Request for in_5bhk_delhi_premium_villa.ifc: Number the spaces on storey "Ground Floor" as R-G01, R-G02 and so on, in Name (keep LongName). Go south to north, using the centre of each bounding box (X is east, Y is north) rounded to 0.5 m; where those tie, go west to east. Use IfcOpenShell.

First a look at what the model holds.

```python
import ifcopenshell
import ifcopenshell.util.element
import ifcopenshell.util.placement

model = ifcopenshell.open("in_5bhk_delhi_premium_villa.ifc")
print(model.schema)
storey = next(s for s in model.by_type("IfcBuildingStorey") if s.Name == "Ground Floor")
spaces = [e for e in ifcopenshell.util.element.get_decomposition(storey) if e.is_a("IfcSpace")]
for e in sorted(spaces, key=lambda e: e.id()):
    origin = ifcopenshell.util.placement.get_local_placement(e.ObjectPlacement)[:3, 3]
    print(e.id(), e.Name, e.LongName, origin.round(2) + 0.0, sep=" | ")
```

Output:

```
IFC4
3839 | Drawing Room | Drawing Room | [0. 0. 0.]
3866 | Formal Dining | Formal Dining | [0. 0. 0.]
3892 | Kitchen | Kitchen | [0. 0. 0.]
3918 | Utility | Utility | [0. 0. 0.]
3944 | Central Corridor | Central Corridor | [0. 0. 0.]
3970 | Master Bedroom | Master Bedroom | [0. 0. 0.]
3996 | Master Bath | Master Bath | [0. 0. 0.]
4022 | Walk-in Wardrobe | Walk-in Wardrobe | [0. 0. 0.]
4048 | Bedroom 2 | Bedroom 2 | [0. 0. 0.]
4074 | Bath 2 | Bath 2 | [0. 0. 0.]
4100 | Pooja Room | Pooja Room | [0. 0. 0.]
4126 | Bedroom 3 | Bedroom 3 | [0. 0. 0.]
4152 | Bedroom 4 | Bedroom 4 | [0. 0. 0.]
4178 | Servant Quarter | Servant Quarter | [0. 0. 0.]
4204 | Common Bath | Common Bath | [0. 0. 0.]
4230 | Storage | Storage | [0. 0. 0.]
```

```python
import ifcopenshell
import ifcopenshell.geom
import ifcopenshell.util.element
import ifcopenshell.util.shape

model = ifcopenshell.open("in_5bhk_delhi_premium_villa.ifc")
settings = ifcopenshell.geom.settings()
settings.set("use-world-coords", True)


def centre(element):
    shape = ifcopenshell.geom.create_shape(settings, element)
    return ifcopenshell.util.shape.get_bbox_centroid(shape.geometry)


storey = next(s for s in model.by_type("IfcBuildingStorey") if s.Name == "Ground Floor")
spaces = [e for e in ifcopenshell.util.element.get_decomposition(storey) if e.is_a("IfcSpace")]

# Insertion points can sit at a corner or the storey origin, so sort by the geometry (in metres).
centres = {e: centre(e) for e in spaces}
spaces.sort(key=lambda e: (round(centres[e][1] / 0.5), centres[e][0]))

for i, e in enumerate(spaces, start=1):
    number = f"R-G{i:02d}"
    e.Name = number
    print(e.id(), number)

model.write("in_5bhk_delhi_premium_villa-out.ifc")
```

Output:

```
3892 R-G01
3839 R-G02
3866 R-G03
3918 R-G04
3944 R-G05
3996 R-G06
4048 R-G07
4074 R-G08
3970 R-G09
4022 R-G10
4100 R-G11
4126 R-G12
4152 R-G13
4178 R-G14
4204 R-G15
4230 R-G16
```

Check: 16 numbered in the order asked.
